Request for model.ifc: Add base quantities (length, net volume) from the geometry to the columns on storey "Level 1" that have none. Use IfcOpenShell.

First a look at what the model holds.

```python
import ifcopenshell
import ifcopenshell.util.element
import ifcopenshell.util.unit

model = ifcopenshell.open("model.ifc")
print(model.schema)
for unit_type in ("LENGTHUNIT", "AREAUNIT", "VOLUMEUNIT"):
    print(unit_type, ifcopenshell.util.unit.calculate_unit_scale(model, unit_type))
storey = next(s for s in model.by_type("IfcBuildingStorey") if s.Name == "Level 1")
columns = [e for e in ifcopenshell.util.element.get_decomposition(storey) if e.is_a("IfcColumn")]
for e in sorted(columns, key=lambda e: e.id()):
    print(e.id(), e.is_a(), e.Name, list(ifcopenshell.util.element.get_psets(e, qtos_only=True)), sep=" | ")
```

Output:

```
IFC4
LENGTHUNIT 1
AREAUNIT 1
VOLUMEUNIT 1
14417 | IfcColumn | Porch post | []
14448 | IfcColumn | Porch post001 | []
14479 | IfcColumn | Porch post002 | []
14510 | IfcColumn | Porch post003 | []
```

```python
import ifcopenshell
import ifcopenshell.api.pset
import ifcopenshell.geom
import ifcopenshell.util.element
import ifcopenshell.util.shape
import ifcopenshell.util.unit

model = ifcopenshell.open("model.ifc")
unit_scale = ifcopenshell.util.unit.calculate_unit_scale(model)
volume_scale = ifcopenshell.util.unit.calculate_unit_scale(model, "VOLUMEUNIT")
settings = ifcopenshell.geom.settings()

storey = next(s for s in model.by_type("IfcBuildingStorey") if s.Name == "Level 1")
columns = [e for e in ifcopenshell.util.element.get_decomposition(storey) if e.is_a("IfcColumn")]

for e in sorted(columns, key=lambda e: e.id()):
    if ifcopenshell.util.element.get_psets(e, qtos_only=True, should_inherit=False):
        continue
    # Geometry comes back in metres, in the element's own axes.
    shape = ifcopenshell.geom.create_shape(settings, e)
    values = {
        "Length": ifcopenshell.util.shape.get_z(shape.geometry) / unit_scale,
        "NetVolume": ifcopenshell.util.shape.get_volume(shape.geometry) / volume_scale,
    }
    qto = ifcopenshell.api.pset.add_qto(model, product=e, name="Qto_ColumnBaseQuantities")
    ifcopenshell.api.pset.edit_qto(model, qto=qto, properties=values)
    print(e.id(), {k: round(v, 3) for k, v in values.items()})

model.write("model_rev.ifc")
```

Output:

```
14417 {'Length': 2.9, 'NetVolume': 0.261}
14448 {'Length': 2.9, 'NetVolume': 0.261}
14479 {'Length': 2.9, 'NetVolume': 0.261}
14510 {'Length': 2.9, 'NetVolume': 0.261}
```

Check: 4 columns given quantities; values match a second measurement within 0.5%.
